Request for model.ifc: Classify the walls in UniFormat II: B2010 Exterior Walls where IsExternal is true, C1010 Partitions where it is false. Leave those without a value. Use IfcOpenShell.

First a look at what the model holds.

```python
import ifcopenshell
import ifcopenshell.util.element

model = ifcopenshell.open("model.ifc")
print(model.schema)
print("classifications:", [c.Name for c in model.by_type("IfcClassification")])
values = [ifcopenshell.util.element.get_pset(e, "Pset_WallCommon", "IsExternal") for e in model.by_type("IfcWall")]
for value in (True, False, None):
    print("IsExternal", value, values.count(value))
```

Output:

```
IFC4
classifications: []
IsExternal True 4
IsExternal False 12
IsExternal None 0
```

```python
import ifcopenshell
import ifcopenshell.api.classification
import ifcopenshell.util.element

model = ifcopenshell.open("model.ifc")

system = ifcopenshell.api.classification.add_classification(model, classification="UniFormat II")

walls = model.by_type("IfcWall")
external = {e: ifcopenshell.util.element.get_pset(e, "Pset_WallCommon", "IsExternal") for e in walls}
for flag, code, name in ((True, "B2010", "Exterior Walls"), (False, "C1010", "Partitions")):
    products = [e for e in walls if external[e] is flag]
    ifcopenshell.api.classification.add_reference(
        model, products=products, classification=system, identification=code, name=name
    )
    print(code, len(products))

model.write("model_updated.ifc")
```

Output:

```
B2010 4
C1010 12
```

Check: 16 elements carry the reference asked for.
